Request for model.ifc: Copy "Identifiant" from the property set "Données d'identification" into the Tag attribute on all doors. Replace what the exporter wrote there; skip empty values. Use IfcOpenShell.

First a look at what the model holds.

```python
import ifcopenshell
import ifcopenshell.util.element

model = ifcopenshell.open("model.ifc")
print(model.schema)
doors = model.by_type("IfcDoor")
print(len(doors), "doors")
for e in doors[:8]:
    source = ifcopenshell.util.element.get_pset(e, "Données d'identification", "Identifiant")
    target = e.Tag
    print(e.id(), repr(source), repr(target), sep=" | ")
```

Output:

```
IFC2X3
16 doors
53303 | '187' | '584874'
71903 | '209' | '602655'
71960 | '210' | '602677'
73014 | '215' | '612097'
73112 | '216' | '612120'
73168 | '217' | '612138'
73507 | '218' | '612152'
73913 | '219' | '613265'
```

```python
import ifcopenshell
import ifcopenshell.util.element

model = ifcopenshell.open("model.ifc")

count = 0
for e in model.by_type("IfcDoor"):
    value = ifcopenshell.util.element.get_pset(e, "Données d'identification", "Identifiant")
    current = e.Tag
    if not value or not value.strip() or current == value:
        continue
    e.Tag = value
    count += 1

print(count, "doors updated")

model.write("model_updated.ifc")
```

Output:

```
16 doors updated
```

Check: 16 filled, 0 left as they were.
